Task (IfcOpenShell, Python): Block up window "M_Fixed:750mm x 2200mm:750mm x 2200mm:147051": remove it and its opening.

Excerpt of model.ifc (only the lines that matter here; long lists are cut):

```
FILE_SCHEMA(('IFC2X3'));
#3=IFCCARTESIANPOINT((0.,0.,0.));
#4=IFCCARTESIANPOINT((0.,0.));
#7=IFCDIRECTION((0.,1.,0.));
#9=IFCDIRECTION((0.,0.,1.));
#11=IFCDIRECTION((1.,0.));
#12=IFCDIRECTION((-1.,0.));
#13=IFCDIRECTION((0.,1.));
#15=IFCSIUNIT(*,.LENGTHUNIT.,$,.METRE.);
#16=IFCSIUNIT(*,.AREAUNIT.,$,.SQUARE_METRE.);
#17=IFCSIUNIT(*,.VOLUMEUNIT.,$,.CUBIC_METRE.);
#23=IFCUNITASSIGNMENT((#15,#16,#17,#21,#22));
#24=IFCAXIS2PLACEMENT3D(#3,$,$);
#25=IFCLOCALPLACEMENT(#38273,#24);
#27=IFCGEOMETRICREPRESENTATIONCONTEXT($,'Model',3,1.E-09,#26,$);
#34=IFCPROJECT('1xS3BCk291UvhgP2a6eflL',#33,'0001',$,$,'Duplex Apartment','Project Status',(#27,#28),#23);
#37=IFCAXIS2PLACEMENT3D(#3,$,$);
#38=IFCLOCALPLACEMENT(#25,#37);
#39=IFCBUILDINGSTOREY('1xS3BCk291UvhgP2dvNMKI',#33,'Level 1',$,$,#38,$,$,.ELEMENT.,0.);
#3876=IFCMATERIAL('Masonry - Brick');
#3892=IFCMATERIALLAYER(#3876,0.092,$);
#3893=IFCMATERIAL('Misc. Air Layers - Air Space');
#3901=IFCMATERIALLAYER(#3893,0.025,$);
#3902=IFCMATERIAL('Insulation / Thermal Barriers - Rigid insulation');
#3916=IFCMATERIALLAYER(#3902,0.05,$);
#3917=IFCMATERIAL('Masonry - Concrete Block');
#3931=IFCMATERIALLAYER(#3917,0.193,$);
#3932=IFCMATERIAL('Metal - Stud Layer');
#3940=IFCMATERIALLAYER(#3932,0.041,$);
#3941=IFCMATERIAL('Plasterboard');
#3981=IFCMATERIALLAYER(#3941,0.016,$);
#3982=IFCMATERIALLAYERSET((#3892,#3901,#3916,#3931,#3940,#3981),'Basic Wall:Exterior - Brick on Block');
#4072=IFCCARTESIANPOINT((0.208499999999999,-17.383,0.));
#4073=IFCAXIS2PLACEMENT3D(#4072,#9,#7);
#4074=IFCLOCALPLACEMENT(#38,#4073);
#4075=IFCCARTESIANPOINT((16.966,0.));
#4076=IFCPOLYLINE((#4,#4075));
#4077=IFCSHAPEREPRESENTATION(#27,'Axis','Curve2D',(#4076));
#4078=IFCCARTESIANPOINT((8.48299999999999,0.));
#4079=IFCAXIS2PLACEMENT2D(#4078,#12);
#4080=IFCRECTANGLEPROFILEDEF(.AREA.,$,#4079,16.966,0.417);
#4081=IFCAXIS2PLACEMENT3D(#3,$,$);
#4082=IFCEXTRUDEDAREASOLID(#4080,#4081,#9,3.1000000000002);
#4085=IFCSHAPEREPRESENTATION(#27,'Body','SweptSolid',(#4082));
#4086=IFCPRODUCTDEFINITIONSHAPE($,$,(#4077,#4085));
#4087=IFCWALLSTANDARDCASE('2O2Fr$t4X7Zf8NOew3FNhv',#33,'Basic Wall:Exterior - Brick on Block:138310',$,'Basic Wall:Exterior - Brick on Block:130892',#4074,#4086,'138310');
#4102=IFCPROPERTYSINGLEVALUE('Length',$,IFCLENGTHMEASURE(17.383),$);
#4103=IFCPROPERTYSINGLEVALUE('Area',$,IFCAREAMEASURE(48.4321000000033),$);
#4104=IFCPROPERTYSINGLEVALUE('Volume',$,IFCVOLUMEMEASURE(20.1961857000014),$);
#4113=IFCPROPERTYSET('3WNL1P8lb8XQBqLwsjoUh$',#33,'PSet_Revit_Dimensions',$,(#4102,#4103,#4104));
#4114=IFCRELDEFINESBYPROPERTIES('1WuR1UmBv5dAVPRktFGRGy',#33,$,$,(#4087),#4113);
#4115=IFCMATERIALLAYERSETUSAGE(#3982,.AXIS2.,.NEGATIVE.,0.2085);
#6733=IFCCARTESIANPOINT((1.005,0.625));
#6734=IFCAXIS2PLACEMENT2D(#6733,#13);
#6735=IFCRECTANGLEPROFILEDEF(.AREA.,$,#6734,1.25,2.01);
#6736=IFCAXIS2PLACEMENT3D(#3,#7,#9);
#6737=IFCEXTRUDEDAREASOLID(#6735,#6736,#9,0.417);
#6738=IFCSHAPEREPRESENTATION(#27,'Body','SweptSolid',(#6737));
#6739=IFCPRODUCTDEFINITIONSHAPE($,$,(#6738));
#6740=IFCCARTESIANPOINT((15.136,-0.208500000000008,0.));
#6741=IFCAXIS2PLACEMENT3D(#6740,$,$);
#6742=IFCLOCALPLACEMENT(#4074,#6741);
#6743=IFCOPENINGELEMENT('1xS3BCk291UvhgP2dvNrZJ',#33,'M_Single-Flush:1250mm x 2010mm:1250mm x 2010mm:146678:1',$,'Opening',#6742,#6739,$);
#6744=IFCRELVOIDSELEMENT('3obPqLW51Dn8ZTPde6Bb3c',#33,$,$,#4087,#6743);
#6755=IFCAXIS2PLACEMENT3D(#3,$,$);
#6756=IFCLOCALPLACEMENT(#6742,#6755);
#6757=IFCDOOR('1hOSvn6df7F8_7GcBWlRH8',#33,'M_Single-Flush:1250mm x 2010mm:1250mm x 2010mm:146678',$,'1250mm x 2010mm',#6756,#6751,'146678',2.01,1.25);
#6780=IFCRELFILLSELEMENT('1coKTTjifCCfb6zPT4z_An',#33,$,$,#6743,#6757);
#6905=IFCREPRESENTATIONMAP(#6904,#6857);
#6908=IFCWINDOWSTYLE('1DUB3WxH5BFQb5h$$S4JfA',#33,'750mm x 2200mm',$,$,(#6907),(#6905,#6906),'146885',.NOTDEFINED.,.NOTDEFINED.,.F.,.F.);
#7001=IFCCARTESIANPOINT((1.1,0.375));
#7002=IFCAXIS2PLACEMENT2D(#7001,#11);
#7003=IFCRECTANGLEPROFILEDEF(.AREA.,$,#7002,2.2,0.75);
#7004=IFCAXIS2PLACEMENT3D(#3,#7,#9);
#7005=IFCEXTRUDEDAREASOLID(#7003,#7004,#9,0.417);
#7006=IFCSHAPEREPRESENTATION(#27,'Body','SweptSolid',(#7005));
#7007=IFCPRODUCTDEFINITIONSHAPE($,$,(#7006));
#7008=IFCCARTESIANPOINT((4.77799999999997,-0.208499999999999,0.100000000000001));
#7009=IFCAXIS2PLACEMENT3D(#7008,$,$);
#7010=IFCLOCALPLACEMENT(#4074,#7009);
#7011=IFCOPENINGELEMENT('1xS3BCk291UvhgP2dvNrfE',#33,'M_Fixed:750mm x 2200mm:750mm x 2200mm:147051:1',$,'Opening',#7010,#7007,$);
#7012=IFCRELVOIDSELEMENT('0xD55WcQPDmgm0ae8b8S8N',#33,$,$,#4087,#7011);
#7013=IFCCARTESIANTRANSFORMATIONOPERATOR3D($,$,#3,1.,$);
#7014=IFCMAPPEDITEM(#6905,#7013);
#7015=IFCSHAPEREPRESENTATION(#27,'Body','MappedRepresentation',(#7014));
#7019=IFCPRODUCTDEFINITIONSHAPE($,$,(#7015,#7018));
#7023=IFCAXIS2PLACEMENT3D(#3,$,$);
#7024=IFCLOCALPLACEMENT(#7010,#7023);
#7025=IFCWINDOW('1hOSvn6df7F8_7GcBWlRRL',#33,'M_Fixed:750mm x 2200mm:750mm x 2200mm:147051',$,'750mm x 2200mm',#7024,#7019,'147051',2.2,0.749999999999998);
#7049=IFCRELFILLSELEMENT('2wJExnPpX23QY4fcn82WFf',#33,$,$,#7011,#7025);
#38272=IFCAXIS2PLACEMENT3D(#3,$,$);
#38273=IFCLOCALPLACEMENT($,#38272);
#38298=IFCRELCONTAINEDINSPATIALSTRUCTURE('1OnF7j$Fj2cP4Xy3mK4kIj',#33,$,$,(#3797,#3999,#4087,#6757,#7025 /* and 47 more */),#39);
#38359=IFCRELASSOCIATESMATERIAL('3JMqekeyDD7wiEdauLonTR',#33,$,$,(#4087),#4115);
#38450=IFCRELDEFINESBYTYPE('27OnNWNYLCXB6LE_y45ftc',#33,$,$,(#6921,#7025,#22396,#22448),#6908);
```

```python
import ifcopenshell
import ifcopenshell.api.feature
import ifcopenshell.api.pset
import ifcopenshell.api.root
import ifcopenshell.geom
import ifcopenshell.util.element
import ifcopenshell.util.shape
import ifcopenshell.util.unit

model = ifcopenshell.open("model.ifc")
area_scale = ifcopenshell.util.unit.calculate_unit_scale(model, "AREAUNIT")
volume_scale = ifcopenshell.util.unit.calculate_unit_scale(model, "VOLUMEUNIT")
settings = ifcopenshell.geom.settings()


def volume(element):
    """Net volume in cubic metres, openings subtracted."""
    shape = ifcopenshell.geom.create_shape(settings, element)
    return ifcopenshell.util.shape.get_volume(shape.geometry)


window = model.by_guid("1hOSvn6df7F8_7GcBWlRRL")
opening = window.FillsVoids[0].RelatingOpeningElement
wall = opening.VoidsElements[0].RelatingBuildingElement
before = volume(wall)

ifcopenshell.api.root.remove_product(model, product=window)
ifcopenshell.api.feature.remove_feature(model, feature=opening)

after = volume(wall)
thickness = 0.417  # wall thickness in metres

# Update the wall's stored quantities.
pset = model.by_id(ifcopenshell.util.element.get_pset(wall, "PSet_Revit_Dimensions", should_inherit=False)["id"])
ifcopenshell.api.pset.edit_pset(model, pset=pset, properties={
    "Area": model.create_entity("IfcAreaMeasure", after / thickness / area_scale),
    "Volume": model.create_entity("IfcVolumeMeasure", after / volume_scale),
})

print(f"wall volume {before:.3f} -> {after:.3f} m3")

model.write("model-out.ifc")
```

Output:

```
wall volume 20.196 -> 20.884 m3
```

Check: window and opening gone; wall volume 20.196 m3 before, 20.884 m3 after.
